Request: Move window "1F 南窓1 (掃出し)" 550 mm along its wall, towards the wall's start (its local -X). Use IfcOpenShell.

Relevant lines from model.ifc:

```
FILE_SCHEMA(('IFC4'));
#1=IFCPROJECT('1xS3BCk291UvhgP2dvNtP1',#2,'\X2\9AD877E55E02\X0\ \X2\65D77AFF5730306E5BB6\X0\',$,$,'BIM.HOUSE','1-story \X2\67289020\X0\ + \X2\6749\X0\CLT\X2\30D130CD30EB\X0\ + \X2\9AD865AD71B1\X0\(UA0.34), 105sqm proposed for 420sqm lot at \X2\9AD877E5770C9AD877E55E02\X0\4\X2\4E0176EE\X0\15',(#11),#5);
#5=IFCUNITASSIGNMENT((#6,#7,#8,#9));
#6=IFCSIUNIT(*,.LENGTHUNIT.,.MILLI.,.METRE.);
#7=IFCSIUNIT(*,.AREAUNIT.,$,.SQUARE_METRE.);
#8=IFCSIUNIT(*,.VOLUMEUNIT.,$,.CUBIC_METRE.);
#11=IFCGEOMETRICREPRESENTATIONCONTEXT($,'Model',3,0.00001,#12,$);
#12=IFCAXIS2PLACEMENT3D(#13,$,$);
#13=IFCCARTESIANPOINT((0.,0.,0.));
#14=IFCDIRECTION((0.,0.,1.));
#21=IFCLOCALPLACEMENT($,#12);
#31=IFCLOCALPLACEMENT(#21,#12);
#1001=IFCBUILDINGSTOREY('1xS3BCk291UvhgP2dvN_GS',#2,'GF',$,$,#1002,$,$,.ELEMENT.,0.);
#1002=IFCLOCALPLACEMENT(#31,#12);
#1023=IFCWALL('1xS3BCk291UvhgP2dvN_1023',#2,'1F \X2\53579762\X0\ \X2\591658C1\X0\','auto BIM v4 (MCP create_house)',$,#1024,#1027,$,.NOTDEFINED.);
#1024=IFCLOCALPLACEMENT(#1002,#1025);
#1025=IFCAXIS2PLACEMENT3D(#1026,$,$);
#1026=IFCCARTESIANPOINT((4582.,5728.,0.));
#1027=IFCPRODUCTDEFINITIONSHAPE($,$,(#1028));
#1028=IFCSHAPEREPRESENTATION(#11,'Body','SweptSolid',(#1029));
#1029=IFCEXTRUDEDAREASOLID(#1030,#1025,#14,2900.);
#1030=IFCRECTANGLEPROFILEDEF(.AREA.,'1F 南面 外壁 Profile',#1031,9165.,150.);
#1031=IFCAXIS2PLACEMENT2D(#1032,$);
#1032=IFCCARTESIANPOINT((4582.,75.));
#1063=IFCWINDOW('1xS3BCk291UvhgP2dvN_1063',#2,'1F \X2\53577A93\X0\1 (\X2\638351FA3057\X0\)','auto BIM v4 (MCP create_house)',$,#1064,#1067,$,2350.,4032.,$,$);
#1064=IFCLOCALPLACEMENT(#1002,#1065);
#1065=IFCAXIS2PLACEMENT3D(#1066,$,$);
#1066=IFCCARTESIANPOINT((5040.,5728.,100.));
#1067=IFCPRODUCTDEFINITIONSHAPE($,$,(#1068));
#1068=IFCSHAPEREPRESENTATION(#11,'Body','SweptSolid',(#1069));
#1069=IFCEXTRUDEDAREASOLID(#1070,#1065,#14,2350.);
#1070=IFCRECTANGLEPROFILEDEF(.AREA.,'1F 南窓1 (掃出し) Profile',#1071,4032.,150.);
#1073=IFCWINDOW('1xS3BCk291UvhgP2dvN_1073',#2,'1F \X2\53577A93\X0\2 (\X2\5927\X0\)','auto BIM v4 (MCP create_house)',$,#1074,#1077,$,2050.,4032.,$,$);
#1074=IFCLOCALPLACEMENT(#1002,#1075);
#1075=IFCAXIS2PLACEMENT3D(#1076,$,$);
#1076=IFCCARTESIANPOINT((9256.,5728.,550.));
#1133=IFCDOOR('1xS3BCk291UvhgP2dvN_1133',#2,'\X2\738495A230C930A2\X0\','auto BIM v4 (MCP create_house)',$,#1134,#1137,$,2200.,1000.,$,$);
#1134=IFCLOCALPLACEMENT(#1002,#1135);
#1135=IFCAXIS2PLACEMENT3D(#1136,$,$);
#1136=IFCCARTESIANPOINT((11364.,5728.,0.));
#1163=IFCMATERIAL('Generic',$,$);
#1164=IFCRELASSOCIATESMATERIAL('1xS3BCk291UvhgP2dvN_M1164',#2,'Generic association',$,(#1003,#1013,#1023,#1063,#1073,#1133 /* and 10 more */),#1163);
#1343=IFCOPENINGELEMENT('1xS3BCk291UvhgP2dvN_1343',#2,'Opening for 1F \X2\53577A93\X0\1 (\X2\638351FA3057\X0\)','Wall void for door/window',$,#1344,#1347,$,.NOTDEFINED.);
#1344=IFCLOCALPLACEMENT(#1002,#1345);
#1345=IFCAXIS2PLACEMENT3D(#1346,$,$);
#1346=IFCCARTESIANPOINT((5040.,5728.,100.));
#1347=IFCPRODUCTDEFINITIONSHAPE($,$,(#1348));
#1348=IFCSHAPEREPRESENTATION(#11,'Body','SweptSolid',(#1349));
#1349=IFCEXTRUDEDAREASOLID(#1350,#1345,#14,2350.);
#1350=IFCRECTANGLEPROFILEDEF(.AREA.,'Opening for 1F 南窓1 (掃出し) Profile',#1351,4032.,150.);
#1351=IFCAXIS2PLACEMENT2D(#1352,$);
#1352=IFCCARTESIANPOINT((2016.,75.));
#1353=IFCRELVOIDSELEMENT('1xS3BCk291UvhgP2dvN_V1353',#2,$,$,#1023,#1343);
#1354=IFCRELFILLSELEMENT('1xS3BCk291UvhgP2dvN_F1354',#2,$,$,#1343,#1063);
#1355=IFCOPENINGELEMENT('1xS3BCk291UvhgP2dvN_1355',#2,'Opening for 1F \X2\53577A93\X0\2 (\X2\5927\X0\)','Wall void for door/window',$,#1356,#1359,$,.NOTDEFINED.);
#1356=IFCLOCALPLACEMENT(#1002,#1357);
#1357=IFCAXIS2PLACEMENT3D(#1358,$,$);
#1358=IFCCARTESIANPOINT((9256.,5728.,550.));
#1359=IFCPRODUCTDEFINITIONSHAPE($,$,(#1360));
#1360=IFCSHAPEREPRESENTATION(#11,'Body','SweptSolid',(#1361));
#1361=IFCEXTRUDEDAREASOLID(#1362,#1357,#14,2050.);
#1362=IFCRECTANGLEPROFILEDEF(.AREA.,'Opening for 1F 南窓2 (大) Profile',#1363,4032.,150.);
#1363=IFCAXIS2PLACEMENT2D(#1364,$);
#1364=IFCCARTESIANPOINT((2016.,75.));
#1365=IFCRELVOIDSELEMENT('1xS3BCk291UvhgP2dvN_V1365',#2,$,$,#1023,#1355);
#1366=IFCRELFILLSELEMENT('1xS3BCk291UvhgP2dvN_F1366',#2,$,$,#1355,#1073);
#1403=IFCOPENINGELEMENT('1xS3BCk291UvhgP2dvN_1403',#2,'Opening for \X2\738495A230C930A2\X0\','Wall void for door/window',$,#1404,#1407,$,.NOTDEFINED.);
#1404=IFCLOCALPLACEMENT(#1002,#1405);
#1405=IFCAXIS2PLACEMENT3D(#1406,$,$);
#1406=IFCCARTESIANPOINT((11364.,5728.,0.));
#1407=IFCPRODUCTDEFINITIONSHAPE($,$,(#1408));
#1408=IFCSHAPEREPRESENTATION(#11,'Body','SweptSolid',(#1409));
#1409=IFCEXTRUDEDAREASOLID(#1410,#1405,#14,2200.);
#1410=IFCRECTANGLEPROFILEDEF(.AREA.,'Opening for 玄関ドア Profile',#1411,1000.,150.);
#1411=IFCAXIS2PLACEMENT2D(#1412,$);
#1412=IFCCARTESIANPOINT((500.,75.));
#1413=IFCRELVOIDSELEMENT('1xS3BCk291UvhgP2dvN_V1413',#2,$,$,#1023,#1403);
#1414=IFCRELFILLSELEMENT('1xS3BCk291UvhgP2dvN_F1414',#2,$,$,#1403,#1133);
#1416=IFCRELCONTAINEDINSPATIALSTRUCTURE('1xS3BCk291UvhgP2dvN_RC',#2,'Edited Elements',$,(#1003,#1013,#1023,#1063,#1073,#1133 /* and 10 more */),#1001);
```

```python
import ifcopenshell
import ifcopenshell.api.geometry
import ifcopenshell.util.placement
import ifcopenshell.util.unit

model = ifcopenshell.open("model.ifc")
unit_scale = ifcopenshell.util.unit.calculate_unit_scale(model)

window = model.by_id(1063)
opening = window.FillsVoids[0].RelatingOpeningElement
wall = opening.VoidsElements[0].RelatingBuildingElement

wall_matrix = ifcopenshell.util.placement.get_local_placement(wall.ObjectPlacement)
shift = wall_matrix[:3, 0] * -0.55 / unit_scale
before = ifcopenshell.util.placement.get_local_placement(window.ObjectPlacement)[:3, 3].copy()

# The window is not placed relative to its opening, so move both.
for product in (opening, window):
    matrix = ifcopenshell.util.placement.get_local_placement(product.ObjectPlacement)
    matrix[:3, 3] += shift
    ifcopenshell.api.geometry.edit_object_placement(model, product=product, matrix=matrix, is_si=False)

after = ifcopenshell.util.placement.get_local_placement(window.ObjectPlacement)[:3, 3]
print("window moved by", (after - before).round(3) + 0.0)

model.write("model-out.ifc")
```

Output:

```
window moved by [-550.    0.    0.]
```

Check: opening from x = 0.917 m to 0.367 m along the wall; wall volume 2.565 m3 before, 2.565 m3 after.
